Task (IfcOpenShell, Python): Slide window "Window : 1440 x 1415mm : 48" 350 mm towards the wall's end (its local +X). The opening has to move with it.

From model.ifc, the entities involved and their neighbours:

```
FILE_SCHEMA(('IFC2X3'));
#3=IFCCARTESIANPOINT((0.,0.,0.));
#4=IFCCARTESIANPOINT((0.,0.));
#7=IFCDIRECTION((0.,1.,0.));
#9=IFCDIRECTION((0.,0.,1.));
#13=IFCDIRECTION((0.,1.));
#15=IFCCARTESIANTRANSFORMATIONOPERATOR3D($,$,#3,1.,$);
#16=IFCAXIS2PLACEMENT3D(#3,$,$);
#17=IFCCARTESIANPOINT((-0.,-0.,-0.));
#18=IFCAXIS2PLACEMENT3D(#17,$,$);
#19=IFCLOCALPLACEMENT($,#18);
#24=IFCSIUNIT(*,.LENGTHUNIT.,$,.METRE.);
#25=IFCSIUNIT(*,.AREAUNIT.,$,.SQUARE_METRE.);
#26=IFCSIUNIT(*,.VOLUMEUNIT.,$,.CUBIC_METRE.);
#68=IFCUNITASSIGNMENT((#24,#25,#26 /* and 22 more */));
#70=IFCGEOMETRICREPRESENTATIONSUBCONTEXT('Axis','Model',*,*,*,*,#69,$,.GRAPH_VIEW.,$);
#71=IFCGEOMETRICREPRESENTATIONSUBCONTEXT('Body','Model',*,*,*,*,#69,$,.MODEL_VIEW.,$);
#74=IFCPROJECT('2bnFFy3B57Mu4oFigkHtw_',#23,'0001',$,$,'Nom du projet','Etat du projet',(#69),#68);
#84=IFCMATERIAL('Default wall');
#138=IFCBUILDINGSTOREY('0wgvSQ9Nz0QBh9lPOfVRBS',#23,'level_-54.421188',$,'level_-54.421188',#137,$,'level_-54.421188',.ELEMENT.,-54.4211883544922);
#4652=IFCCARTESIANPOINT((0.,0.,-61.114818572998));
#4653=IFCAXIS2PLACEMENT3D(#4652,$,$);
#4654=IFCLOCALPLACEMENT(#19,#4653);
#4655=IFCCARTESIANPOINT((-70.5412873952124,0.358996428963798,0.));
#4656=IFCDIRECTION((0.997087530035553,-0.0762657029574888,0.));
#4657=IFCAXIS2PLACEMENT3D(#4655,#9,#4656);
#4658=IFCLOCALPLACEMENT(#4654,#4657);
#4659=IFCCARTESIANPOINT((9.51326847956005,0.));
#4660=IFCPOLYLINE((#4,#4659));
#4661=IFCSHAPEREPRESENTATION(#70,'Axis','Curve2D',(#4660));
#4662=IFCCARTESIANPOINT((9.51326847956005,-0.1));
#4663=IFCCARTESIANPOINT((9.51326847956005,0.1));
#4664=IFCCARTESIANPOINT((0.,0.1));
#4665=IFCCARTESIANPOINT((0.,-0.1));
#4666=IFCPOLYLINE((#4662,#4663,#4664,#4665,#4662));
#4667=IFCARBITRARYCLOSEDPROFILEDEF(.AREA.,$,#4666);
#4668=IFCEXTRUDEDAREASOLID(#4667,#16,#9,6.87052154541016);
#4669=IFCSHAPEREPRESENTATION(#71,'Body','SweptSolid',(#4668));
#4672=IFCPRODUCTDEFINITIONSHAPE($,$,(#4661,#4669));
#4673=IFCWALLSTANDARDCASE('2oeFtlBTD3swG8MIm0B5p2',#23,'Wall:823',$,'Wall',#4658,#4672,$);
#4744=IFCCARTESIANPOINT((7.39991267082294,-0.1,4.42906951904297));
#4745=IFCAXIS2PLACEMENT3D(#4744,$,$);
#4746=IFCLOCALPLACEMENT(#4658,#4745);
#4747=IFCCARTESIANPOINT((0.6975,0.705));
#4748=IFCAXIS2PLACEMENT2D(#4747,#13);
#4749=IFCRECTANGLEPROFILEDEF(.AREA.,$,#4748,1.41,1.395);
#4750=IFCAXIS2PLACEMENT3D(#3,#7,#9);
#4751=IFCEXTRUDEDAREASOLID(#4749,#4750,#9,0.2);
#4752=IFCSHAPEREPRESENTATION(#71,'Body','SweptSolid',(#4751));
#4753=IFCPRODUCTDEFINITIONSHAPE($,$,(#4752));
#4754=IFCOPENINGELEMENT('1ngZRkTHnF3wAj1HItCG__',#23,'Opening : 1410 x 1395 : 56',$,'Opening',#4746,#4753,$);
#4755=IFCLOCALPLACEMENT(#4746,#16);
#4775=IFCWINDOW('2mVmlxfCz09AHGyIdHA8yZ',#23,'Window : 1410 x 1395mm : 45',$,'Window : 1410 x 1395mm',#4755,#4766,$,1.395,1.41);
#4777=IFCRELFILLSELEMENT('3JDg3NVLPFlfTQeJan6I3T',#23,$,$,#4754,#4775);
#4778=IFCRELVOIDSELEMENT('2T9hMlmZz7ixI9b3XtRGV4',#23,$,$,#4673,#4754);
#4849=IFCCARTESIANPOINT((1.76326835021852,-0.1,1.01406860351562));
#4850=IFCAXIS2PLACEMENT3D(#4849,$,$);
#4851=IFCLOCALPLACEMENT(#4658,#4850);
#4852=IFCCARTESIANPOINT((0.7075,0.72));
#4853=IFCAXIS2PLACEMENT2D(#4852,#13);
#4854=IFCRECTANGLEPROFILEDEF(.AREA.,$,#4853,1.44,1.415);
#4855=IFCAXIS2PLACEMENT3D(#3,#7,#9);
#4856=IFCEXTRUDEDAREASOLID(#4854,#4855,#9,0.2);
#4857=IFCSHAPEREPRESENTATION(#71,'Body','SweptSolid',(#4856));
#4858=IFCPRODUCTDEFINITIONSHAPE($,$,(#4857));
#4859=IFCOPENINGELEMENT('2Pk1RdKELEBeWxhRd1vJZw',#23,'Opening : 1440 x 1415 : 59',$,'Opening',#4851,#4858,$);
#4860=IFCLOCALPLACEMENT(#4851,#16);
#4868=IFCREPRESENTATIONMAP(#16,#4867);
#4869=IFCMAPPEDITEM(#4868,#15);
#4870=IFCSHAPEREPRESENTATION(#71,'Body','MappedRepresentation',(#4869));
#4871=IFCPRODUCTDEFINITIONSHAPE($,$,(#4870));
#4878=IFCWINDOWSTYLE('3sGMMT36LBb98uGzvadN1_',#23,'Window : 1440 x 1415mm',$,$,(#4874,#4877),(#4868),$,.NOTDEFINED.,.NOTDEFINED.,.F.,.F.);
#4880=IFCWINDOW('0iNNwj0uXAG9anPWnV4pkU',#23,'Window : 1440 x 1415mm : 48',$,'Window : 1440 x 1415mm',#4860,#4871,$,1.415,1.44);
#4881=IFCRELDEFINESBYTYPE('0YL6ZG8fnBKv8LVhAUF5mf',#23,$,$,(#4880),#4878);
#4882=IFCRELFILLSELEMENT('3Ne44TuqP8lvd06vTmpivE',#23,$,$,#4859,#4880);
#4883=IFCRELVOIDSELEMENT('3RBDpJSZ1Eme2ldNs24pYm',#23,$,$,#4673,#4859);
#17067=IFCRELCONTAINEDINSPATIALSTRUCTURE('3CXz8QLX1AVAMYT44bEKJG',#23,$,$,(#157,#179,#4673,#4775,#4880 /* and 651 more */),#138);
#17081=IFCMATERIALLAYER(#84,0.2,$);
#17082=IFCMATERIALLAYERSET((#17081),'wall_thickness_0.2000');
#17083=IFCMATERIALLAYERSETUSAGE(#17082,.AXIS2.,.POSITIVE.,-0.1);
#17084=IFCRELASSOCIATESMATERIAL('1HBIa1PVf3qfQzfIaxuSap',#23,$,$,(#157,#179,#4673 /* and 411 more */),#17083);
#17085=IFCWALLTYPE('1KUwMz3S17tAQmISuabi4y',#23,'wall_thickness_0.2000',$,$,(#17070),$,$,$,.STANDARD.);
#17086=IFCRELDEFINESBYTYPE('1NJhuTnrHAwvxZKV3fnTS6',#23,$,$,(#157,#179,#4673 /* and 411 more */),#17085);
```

```python
import ifcopenshell
import ifcopenshell.api.geometry
import ifcopenshell.util.placement
import ifcopenshell.util.unit

model = ifcopenshell.open("model.ifc")
unit_scale = ifcopenshell.util.unit.calculate_unit_scale(model)

window = model.by_id(4880)
opening = window.FillsVoids[0].RelatingOpeningElement
wall = opening.VoidsElements[0].RelatingBuildingElement

wall_matrix = ifcopenshell.util.placement.get_local_placement(wall.ObjectPlacement)
shift = wall_matrix[:3, 0] * 0.35 / unit_scale
before = ifcopenshell.util.placement.get_local_placement(window.ObjectPlacement)[:3, 3].copy()

# The window is placed relative to its opening, so it follows when the opening moves.
matrix = ifcopenshell.util.placement.get_local_placement(opening.ObjectPlacement)
matrix[:3, 3] += shift
ifcopenshell.api.geometry.edit_object_placement(
    model, product=opening, matrix=matrix, is_si=False, should_transform_children=True
)

after = ifcopenshell.util.placement.get_local_placement(window.ObjectPlacement)[:3, 3]
print("window moved by", (after - before).round(3) + 0.0)

model.write("model-out.ifc")
```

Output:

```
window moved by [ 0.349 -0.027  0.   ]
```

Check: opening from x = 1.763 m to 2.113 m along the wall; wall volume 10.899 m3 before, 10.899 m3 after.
